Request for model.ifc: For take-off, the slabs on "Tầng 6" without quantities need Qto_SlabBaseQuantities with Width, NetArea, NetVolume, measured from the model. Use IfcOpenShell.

First a look at what the model holds.

```python
import ifcopenshell
import ifcopenshell.util.element
import ifcopenshell.util.unit

model = ifcopenshell.open("model.ifc")
print(model.schema)
for unit_type in ("LENGTHUNIT", "AREAUNIT", "VOLUMEUNIT"):
    print(unit_type, ifcopenshell.util.unit.calculate_unit_scale(model, unit_type))
storey = next(s for s in model.by_type("IfcBuildingStorey") if s.Name == "Tầng 6")
slabs = [e for e in ifcopenshell.util.element.get_decomposition(storey) if e.is_a("IfcSlab")]
for e in sorted(slabs, key=lambda e: e.id()):
    print(e.id(), e.is_a(), e.Name, list(ifcopenshell.util.element.get_psets(e, qtos_only=True)), sep=" | ")
```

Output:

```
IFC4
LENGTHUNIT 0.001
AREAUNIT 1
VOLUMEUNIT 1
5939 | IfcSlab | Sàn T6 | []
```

```python
import ifcopenshell
import ifcopenshell.api.pset
import ifcopenshell.geom
import ifcopenshell.util.element
import ifcopenshell.util.shape
import ifcopenshell.util.unit

model = ifcopenshell.open("model.ifc")
unit_scale = ifcopenshell.util.unit.calculate_unit_scale(model)
area_scale = ifcopenshell.util.unit.calculate_unit_scale(model, "AREAUNIT")
volume_scale = ifcopenshell.util.unit.calculate_unit_scale(model, "VOLUMEUNIT")
settings = ifcopenshell.geom.settings()

storey = next(s for s in model.by_type("IfcBuildingStorey") if s.Name == "Tầng 6")
slabs = [e for e in ifcopenshell.util.element.get_decomposition(storey) if e.is_a("IfcSlab")]

for e in sorted(slabs, key=lambda e: e.id()):
    if ifcopenshell.util.element.get_psets(e, qtos_only=True, should_inherit=False):
        continue
    # Geometry comes back in metres, in the element's own axes.
    shape = ifcopenshell.geom.create_shape(settings, e)
    values = {
        "Width": ifcopenshell.util.shape.get_z(shape.geometry) / unit_scale,
        "NetArea": ifcopenshell.util.shape.get_footprint_area(shape.geometry) / area_scale,
        "NetVolume": ifcopenshell.util.shape.get_volume(shape.geometry) / volume_scale,
    }
    qto = ifcopenshell.api.pset.add_qto(model, product=e, name="Qto_SlabBaseQuantities")
    ifcopenshell.api.pset.edit_qto(model, qto=qto, properties=values)
    print(e.id(), {k: round(v, 3) for k, v in values.items()})

model.write("model-out.ifc")
```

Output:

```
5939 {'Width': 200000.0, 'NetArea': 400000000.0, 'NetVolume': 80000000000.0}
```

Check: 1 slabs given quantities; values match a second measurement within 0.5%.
